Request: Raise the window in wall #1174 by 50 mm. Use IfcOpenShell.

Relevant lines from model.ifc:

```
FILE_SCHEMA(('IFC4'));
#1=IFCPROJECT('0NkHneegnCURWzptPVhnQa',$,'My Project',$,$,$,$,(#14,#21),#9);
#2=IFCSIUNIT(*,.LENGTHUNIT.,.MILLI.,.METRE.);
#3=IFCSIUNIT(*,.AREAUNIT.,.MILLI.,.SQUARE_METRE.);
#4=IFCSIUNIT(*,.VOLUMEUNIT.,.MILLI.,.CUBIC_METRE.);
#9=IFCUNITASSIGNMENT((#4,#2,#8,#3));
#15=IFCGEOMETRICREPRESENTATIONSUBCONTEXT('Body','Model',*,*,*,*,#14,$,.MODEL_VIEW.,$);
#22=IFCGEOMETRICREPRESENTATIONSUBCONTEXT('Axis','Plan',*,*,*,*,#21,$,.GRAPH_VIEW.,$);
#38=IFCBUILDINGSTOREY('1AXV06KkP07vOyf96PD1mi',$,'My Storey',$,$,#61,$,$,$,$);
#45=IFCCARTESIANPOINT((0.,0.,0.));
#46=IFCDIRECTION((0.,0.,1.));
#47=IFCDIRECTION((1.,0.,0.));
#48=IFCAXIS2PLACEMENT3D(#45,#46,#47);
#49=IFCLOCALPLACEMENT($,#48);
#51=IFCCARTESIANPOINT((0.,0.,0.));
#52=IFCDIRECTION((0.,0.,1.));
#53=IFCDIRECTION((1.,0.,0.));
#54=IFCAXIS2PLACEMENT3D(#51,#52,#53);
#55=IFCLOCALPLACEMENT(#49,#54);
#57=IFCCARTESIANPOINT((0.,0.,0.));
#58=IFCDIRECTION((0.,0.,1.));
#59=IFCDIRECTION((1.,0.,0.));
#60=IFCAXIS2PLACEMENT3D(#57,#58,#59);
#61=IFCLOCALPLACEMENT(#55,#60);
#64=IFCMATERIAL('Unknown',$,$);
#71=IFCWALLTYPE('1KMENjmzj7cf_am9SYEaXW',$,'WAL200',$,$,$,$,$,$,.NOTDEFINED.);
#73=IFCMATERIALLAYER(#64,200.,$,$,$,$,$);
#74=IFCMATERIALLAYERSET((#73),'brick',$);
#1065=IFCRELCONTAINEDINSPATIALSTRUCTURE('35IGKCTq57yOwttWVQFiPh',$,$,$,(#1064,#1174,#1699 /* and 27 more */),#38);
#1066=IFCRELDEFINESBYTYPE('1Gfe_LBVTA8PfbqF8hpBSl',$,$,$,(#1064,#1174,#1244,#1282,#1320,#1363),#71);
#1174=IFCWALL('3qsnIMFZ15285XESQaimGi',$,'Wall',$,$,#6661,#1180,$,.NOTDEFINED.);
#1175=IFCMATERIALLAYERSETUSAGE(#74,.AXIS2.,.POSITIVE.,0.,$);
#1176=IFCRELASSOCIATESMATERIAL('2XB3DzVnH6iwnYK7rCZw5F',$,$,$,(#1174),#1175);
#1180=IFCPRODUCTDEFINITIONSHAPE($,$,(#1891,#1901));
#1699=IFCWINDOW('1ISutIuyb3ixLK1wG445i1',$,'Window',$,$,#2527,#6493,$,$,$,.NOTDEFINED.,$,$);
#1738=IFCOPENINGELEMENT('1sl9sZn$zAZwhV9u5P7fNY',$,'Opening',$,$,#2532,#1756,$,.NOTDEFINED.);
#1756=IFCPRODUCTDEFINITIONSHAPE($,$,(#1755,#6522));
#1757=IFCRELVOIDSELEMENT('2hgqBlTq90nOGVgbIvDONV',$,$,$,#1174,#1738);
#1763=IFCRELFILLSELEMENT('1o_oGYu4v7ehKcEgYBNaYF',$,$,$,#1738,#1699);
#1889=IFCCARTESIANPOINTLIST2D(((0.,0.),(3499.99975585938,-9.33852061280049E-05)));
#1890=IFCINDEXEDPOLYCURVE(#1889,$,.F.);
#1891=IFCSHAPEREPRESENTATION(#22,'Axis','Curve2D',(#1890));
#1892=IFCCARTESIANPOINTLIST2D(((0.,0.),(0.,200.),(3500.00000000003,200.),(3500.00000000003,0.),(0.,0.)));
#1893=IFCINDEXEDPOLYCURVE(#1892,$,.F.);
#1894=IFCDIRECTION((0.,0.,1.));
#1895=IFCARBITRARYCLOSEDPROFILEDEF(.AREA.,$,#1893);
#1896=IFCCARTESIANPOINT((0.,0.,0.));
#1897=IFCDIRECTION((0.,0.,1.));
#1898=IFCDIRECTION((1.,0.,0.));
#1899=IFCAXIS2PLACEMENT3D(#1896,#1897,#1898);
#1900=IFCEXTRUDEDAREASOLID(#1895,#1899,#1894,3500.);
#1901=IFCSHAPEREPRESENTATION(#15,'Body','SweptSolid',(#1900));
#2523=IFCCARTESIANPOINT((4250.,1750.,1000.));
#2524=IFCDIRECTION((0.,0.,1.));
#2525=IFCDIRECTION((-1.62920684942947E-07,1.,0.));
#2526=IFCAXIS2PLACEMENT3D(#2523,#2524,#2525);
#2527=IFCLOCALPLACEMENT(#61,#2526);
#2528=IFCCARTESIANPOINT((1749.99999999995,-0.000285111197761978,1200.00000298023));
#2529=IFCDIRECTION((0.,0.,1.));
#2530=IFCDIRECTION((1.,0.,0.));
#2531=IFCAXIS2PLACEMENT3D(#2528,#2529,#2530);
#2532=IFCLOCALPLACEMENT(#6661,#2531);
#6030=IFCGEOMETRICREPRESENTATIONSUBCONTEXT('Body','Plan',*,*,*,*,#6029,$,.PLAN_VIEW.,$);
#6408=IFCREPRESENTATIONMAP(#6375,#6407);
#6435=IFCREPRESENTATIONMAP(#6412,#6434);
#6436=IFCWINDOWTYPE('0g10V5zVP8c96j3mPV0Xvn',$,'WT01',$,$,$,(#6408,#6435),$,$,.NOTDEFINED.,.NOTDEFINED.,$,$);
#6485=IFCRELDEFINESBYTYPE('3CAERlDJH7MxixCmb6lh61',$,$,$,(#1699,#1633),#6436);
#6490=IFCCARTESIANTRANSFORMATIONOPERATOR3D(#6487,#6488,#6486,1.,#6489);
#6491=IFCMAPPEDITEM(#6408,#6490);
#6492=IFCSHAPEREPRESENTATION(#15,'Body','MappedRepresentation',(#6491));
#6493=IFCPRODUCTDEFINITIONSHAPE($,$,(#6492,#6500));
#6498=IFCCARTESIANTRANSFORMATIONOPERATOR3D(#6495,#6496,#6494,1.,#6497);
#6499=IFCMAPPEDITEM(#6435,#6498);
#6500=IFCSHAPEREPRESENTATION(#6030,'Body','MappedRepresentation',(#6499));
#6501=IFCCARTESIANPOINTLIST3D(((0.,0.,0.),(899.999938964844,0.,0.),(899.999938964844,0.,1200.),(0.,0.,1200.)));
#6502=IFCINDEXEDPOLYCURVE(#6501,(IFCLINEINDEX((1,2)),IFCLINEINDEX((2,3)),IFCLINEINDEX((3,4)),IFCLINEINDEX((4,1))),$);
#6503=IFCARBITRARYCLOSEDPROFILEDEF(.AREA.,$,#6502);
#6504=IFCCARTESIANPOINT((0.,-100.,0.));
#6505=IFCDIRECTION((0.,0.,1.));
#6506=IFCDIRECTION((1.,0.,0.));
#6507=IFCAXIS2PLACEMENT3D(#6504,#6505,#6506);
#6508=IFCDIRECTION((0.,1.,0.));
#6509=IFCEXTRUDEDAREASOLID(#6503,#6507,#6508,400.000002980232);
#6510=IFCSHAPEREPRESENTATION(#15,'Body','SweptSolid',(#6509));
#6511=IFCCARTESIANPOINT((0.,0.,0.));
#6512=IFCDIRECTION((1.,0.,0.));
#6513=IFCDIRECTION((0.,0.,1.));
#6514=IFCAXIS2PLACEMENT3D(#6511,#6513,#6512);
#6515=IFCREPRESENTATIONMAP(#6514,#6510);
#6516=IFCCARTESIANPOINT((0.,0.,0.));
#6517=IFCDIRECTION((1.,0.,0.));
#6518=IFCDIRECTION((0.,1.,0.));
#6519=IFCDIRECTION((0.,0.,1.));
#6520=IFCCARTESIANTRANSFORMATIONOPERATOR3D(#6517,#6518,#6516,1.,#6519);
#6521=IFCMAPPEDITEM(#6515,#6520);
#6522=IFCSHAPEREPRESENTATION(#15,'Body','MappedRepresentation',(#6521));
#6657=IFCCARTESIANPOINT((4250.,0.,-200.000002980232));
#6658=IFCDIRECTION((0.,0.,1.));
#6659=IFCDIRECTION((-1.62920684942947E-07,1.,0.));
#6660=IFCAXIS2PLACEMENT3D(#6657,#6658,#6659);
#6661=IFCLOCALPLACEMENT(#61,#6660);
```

```python
import numpy as np
import ifcopenshell
import ifcopenshell.api.geometry
import ifcopenshell.util.placement
import ifcopenshell.util.unit

model = ifcopenshell.open("model.ifc")
unit_scale = ifcopenshell.util.unit.calculate_unit_scale(model)

window = model.by_id(1699)
opening = window.FillsVoids[0].RelatingOpeningElement
dz = 50.0

shift = np.array([0.0, 0.0, dz])
# The window is not placed relative to its opening, so move both.
for product in (opening, window):
    matrix = ifcopenshell.util.placement.get_local_placement(product.ObjectPlacement)
    matrix[:3, 3] += shift
    ifcopenshell.api.geometry.edit_object_placement(model, product=product, matrix=matrix, is_si=False)

print(f"moved by {dz * unit_scale:+.3f} m")

model.write("model_v2.ifc")
```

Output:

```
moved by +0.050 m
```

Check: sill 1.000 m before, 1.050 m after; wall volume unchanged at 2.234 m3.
